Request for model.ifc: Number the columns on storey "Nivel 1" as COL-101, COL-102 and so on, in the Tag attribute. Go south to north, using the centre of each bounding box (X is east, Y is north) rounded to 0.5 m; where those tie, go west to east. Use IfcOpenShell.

First a look at what the model holds.

```python
import ifcopenshell
import ifcopenshell.util.element
import ifcopenshell.util.placement

model = ifcopenshell.open("model.ifc")
print(model.schema)
storey = next(s for s in model.by_type("IfcBuildingStorey") if s.Name == "Nivel 1")
columns = [e for e in ifcopenshell.util.element.get_decomposition(storey) if e.is_a("IfcColumn")]
for e in sorted(columns, key=lambda e: e.id()):
    origin = ifcopenshell.util.placement.get_local_placement(e.ObjectPlacement)[:3, 3]
    print(e.id(), e.Tag, e.Name, origin.round(2) + 0.0, sep=" | ")
```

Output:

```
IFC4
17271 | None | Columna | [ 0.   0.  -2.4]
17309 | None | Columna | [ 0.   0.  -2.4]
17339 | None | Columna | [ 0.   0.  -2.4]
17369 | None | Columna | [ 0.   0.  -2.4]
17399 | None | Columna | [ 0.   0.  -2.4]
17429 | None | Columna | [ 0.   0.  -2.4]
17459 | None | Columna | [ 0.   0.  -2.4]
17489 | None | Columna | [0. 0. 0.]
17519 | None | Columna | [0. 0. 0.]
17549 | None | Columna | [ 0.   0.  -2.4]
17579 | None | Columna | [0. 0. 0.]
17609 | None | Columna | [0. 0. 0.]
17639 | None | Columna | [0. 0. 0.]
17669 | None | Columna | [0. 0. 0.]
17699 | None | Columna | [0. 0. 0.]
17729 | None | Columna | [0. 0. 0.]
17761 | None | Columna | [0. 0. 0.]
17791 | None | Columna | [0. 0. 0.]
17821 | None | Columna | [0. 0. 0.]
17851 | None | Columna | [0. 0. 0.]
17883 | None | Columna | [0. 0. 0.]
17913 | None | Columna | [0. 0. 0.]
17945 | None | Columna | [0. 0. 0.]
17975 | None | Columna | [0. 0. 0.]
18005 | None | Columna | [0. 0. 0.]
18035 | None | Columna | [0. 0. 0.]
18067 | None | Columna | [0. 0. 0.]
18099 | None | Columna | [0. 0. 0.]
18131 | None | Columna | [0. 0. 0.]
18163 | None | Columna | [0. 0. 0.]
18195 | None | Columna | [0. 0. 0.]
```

```python
import ifcopenshell
import ifcopenshell.geom
import ifcopenshell.util.element
import ifcopenshell.util.shape

model = ifcopenshell.open("model.ifc")
settings = ifcopenshell.geom.settings()
settings.set("use-world-coords", True)


def centre(element):
    shape = ifcopenshell.geom.create_shape(settings, element)
    return ifcopenshell.util.shape.get_bbox_centroid(shape.geometry)


storey = next(s for s in model.by_type("IfcBuildingStorey") if s.Name == "Nivel 1")
columns = [e for e in ifcopenshell.util.element.get_decomposition(storey) if e.is_a("IfcColumn")]

# Insertion points can sit at a corner or the storey origin, so sort by the geometry (in metres).
centres = {e: centre(e) for e in columns}
columns.sort(key=lambda e: (round(centres[e][1] / 0.5), centres[e][0]))

for i, e in enumerate(columns, start=1):
    number = f"COL-1{i:02d}"
    e.Tag = number
    print(e.id(), number)

model.write("model_v2.ifc")
```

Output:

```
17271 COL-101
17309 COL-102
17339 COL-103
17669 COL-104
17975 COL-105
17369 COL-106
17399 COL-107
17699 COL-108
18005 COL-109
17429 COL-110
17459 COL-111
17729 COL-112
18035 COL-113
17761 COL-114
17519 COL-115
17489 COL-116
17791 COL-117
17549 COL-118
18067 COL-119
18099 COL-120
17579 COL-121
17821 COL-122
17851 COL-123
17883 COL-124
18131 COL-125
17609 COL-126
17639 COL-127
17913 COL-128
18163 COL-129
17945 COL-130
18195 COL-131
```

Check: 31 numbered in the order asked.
